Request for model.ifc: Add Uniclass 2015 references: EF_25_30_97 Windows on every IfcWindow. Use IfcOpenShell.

First a look at what the model holds.

```python
import ifcopenshell

model = ifcopenshell.open("model.ifc")
print(model.schema)
print("classifications:", [c.Name for c in model.by_type("IfcClassification")])
for ifc_class in ("IfcDoor", "IfcRoof", "IfcStair", "IfcWall", "IfcWindow"):
    print(ifc_class, len(model.by_type(ifc_class)))
```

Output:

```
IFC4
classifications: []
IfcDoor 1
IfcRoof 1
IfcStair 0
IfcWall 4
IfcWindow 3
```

```python
import ifcopenshell
import ifcopenshell.api.classification

model = ifcopenshell.open("model.ifc")

system = ifcopenshell.api.classification.add_classification(model, classification="Uniclass 2015")

codes = {
    "IfcWindow": ("EF_25_30_97", "Windows"),
}
for ifc_class, (code, name) in codes.items():
    products = model.by_type(ifc_class)
    ifcopenshell.api.classification.add_reference(
        model, products=products, classification=system, identification=code, name=name
    )
    print(code, len(products))

model.write("model-out.ifc")
```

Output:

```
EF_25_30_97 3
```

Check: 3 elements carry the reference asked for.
